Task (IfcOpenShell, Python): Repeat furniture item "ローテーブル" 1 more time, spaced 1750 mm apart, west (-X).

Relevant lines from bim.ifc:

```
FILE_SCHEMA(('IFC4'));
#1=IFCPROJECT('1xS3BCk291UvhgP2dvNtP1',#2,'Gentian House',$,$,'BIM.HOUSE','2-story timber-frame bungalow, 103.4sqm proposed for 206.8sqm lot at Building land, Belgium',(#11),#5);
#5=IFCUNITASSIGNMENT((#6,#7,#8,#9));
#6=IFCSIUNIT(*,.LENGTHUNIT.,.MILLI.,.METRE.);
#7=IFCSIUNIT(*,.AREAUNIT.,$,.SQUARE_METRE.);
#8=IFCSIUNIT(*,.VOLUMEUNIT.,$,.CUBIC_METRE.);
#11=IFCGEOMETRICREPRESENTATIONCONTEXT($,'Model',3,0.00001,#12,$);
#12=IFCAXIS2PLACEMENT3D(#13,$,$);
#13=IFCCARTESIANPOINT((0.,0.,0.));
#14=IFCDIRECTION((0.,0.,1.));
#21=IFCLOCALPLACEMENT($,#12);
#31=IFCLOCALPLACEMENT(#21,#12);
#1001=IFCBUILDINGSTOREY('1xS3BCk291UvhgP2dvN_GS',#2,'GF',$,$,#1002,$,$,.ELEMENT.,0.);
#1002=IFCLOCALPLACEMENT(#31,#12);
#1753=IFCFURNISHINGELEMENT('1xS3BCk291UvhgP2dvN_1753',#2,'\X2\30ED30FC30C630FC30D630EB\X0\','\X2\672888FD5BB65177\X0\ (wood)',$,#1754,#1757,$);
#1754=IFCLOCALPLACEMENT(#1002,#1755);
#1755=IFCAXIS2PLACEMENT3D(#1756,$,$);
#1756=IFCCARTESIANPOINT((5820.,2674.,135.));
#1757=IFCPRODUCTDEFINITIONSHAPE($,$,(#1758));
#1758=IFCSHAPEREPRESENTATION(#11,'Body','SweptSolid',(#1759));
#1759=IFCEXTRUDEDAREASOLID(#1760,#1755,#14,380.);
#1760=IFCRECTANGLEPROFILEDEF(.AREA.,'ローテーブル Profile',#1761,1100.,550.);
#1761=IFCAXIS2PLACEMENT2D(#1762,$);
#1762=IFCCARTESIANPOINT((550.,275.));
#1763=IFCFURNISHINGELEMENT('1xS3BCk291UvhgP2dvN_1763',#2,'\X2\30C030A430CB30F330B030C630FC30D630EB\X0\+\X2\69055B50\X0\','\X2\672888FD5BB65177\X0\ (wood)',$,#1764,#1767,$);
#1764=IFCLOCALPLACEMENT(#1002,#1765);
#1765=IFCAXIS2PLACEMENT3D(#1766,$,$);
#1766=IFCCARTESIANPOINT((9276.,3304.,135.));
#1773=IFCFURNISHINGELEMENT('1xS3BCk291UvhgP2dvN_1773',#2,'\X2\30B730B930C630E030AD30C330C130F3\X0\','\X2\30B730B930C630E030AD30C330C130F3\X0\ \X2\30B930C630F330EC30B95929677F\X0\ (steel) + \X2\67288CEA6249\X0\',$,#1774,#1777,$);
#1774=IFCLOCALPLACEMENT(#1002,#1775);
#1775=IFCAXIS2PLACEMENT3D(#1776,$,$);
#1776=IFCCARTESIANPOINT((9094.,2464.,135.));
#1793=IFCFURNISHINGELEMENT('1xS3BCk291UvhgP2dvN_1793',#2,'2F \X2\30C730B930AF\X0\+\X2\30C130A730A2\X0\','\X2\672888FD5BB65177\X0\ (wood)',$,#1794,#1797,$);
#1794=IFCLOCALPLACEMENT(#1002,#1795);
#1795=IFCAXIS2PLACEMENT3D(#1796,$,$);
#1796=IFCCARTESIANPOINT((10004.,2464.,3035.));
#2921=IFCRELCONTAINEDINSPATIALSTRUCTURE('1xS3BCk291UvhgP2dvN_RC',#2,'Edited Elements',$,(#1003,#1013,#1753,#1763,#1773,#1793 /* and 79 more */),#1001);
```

```python
import numpy as np
import ifcopenshell
import ifcopenshell.api.geometry
import ifcopenshell.api.root
import ifcopenshell.util.element
import ifcopenshell.util.placement
import ifcopenshell.util.unit

model = ifcopenshell.open("bim.ifc")
unit_scale = ifcopenshell.util.unit.calculate_unit_scale(model)


def reuse_history(source, copy):
    """copy_class also copies each property set's owner history, people and application; keep the originals."""
    for rel in copy.IsDefinedBy:
        if rel.is_a("IfcRelDefinesByProperties") and (history := rel.RelatingPropertyDefinition.OwnerHistory):
            rel.RelatingPropertyDefinition.OwnerHistory = source.OwnerHistory
            ifcopenshell.util.element.remove_deep2(model, history)


source = model.by_guid("1xS3BCk291UvhgP2dvN_1753")
base = ifcopenshell.util.placement.get_local_placement(source.ObjectPlacement)
step = np.array([-1.0, 0.0, 0.0]) * 1.75 / unit_scale

for i in range(1, 2):
    copy = ifcopenshell.api.root.copy_class(model, product=source)
    copy.Representation = ifcopenshell.util.element.copy_deep(
        model, source.Representation, exclude=["IfcGeometricRepresentationContext", "IfcRepresentationMap"]
    )
    reuse_history(source, copy)
    matrix = base.copy()
    matrix[:3, 3] += i * step
    print("added at", matrix[:3, 3].round(3) + 0.0)
    ifcopenshell.api.geometry.edit_object_placement(model, product=copy, matrix=matrix, is_si=False)

model.write("bim_rev.ifc")
```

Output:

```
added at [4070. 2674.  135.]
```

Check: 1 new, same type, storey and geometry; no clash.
